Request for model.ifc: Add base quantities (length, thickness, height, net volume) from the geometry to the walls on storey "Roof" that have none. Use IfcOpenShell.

First a look at what the model holds.

```python
import ifcopenshell
import ifcopenshell.util.element
import ifcopenshell.util.unit

model = ifcopenshell.open("model.ifc")
print(model.schema)
for unit_type in ("LENGTHUNIT", "AREAUNIT", "VOLUMEUNIT"):
    print(unit_type, ifcopenshell.util.unit.calculate_unit_scale(model, unit_type))
storey = next(s for s in model.by_type("IfcBuildingStorey") if s.Name == "Roof")
walls = [e for e in ifcopenshell.util.element.get_decomposition(storey) if e.is_a("IfcWall")]
for e in sorted(walls, key=lambda e: e.id()):
    print(e.id(), e.is_a(), e.Name, list(ifcopenshell.util.element.get_psets(e, qtos_only=True)), sep=" | ")
```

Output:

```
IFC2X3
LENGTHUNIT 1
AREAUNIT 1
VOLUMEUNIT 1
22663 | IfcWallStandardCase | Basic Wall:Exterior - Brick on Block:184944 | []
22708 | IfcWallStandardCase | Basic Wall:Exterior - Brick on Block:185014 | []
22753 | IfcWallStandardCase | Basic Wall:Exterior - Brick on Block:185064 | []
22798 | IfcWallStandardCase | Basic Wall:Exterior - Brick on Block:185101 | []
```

```python
import ifcopenshell
import ifcopenshell.api.pset
import ifcopenshell.geom
import ifcopenshell.util.element
import ifcopenshell.util.shape
import ifcopenshell.util.unit

model = ifcopenshell.open("model.ifc")
unit_scale = ifcopenshell.util.unit.calculate_unit_scale(model)
volume_scale = ifcopenshell.util.unit.calculate_unit_scale(model, "VOLUMEUNIT")
settings = ifcopenshell.geom.settings()

storey = next(s for s in model.by_type("IfcBuildingStorey") if s.Name == "Roof")
walls = [e for e in ifcopenshell.util.element.get_decomposition(storey) if e.is_a("IfcWall")]

for e in sorted(walls, key=lambda e: e.id()):
    if ifcopenshell.util.element.get_psets(e, qtos_only=True, should_inherit=False):
        continue
    # Geometry comes back in metres, in the element's own axes.
    shape = ifcopenshell.geom.create_shape(settings, e)
    values = {
        "Length": ifcopenshell.util.shape.get_x(shape.geometry) / unit_scale,
        "Width": ifcopenshell.util.shape.get_y(shape.geometry) / unit_scale,
        "Height": ifcopenshell.util.shape.get_z(shape.geometry) / unit_scale,
        "NetVolume": ifcopenshell.util.shape.get_volume(shape.geometry) / volume_scale,
    }
    qto = ifcopenshell.api.pset.add_qto(model, product=e, name="BaseQuantities")
    ifcopenshell.api.pset.edit_qto(model, qto=qto, properties=values)
    print(e.id(), {k: round(v, 3) for k, v in values.items()})

model.write("model_edited.ifc")
```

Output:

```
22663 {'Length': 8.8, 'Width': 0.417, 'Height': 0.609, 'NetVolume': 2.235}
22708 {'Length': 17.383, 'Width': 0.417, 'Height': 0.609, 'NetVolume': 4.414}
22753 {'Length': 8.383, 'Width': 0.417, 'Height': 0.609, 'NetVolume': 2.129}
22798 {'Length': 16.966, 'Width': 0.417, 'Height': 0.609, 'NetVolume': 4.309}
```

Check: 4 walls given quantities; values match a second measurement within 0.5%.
